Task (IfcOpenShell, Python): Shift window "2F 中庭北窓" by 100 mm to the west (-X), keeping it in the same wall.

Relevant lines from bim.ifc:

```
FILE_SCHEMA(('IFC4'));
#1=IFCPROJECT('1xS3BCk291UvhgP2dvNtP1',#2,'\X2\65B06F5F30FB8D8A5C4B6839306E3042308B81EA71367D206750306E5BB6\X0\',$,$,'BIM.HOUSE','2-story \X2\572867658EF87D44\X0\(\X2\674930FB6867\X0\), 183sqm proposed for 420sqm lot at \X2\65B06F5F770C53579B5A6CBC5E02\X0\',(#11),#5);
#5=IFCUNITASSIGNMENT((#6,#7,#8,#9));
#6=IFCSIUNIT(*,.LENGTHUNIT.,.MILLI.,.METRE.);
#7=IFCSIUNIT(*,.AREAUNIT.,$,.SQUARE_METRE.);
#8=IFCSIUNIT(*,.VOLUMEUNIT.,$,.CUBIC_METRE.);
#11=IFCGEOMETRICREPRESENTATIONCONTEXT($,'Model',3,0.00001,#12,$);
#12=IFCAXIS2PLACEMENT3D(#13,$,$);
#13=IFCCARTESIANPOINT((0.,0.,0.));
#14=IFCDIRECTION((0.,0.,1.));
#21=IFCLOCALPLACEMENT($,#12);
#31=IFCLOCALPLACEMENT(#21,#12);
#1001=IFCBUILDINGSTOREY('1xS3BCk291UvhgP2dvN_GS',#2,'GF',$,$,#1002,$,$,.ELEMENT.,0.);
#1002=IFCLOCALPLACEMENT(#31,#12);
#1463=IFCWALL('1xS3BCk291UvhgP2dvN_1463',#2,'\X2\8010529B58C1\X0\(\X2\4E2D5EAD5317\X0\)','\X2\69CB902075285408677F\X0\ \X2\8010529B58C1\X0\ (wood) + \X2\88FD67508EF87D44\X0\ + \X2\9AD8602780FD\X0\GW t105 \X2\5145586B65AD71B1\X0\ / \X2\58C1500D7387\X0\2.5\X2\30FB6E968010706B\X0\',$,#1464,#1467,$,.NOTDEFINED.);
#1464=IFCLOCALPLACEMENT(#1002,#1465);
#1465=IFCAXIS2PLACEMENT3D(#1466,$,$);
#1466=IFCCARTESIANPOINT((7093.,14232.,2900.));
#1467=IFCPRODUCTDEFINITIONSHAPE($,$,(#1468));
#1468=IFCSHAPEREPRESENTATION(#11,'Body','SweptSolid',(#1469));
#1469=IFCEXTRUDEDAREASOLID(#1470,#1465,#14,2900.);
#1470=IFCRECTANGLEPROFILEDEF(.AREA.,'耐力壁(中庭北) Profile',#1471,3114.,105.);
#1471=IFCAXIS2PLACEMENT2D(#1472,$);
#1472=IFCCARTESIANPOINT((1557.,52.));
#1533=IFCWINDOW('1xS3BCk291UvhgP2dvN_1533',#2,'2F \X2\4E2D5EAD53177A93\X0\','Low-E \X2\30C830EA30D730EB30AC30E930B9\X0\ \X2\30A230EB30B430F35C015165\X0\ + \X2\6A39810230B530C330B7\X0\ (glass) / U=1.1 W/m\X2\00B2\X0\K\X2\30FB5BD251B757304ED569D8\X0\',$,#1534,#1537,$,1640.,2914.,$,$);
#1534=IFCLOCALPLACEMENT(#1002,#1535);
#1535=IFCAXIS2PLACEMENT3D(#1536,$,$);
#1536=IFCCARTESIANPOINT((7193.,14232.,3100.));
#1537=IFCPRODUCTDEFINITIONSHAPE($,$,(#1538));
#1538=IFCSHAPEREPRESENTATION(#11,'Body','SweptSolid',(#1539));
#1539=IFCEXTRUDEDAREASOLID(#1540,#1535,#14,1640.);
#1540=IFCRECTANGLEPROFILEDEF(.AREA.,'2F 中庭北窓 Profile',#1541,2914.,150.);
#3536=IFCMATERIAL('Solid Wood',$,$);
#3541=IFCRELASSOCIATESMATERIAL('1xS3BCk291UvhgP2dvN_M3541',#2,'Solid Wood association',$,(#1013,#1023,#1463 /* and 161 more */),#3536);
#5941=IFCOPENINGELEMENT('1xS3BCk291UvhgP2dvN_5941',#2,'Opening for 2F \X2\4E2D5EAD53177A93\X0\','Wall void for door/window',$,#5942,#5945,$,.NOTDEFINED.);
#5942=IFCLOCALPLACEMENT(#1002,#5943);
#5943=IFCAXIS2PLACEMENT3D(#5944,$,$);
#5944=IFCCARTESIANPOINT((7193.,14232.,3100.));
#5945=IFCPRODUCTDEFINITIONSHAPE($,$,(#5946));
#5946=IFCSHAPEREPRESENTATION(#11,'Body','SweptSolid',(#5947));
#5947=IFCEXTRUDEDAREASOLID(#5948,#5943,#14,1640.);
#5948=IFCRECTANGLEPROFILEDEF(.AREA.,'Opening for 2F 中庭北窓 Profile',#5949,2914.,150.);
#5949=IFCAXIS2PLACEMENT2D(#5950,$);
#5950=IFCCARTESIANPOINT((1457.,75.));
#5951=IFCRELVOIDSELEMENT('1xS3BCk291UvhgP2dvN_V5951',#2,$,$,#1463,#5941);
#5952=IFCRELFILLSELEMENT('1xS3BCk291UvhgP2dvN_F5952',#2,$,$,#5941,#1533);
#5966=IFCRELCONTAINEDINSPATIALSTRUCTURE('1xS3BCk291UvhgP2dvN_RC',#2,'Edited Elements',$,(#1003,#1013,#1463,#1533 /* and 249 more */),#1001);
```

```python
import ifcopenshell
import ifcopenshell.api.geometry
import ifcopenshell.util.placement

model = ifcopenshell.open("bim.ifc")

window = model.by_guid("1xS3BCk291UvhgP2dvN_1533")
opening = window.FillsVoids[0].RelatingOpeningElement
wall = opening.VoidsElements[0].RelatingBuildingElement

wall_matrix = ifcopenshell.util.placement.get_local_placement(wall.ObjectPlacement)
shift = wall_matrix[:3, 0] * -100.0
before = ifcopenshell.util.placement.get_local_placement(window.ObjectPlacement)[:3, 3].copy()

# The window is not placed relative to its opening, so move both.
for product in (opening, window):
    matrix = ifcopenshell.util.placement.get_local_placement(product.ObjectPlacement)
    matrix[:3, 3] += shift
    ifcopenshell.api.geometry.edit_object_placement(model, product=product, matrix=matrix, is_si=False)

after = ifcopenshell.util.placement.get_local_placement(window.ObjectPlacement)[:3, 3]
print("window moved by", (after - before).round(3) + 0.0)

model.write("bim_v2.ifc")
```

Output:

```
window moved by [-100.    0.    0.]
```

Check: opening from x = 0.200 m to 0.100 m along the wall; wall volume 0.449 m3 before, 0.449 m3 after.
